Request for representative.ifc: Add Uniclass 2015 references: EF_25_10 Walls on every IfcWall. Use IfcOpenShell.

First a look at what the model holds.

```python
import ifcopenshell

model = ifcopenshell.open("representative.ifc")
print(model.schema)
print("classifications:", [c.Name for c in model.by_type("IfcClassification")])
for ifc_class in ("IfcDoor", "IfcRoof", "IfcStair", "IfcWall", "IfcWindow"):
    print(ifc_class, len(model.by_type(ifc_class)))
```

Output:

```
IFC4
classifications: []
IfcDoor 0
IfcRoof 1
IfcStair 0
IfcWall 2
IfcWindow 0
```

```python
import ifcopenshell
import ifcopenshell.api.classification

model = ifcopenshell.open("representative.ifc")

system = ifcopenshell.api.classification.add_classification(model, classification="Uniclass 2015")

codes = {
    "IfcWall": ("EF_25_10", "Walls"),
}
for ifc_class, (code, name) in codes.items():
    products = model.by_type(ifc_class)
    ifcopenshell.api.classification.add_reference(
        model, products=products, classification=system, identification=code, name=name
    )
    print(code, len(products))

model.write("representative_edited.ifc")
```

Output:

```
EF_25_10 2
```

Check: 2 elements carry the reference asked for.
